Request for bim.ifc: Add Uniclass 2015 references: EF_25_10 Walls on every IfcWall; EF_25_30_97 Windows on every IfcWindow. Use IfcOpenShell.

First a look at what the model holds.

```python
import ifcopenshell

model = ifcopenshell.open("bim.ifc")
print(model.schema)
print("classifications:", [c.Name for c in model.by_type("IfcClassification")])
for ifc_class in ("IfcDoor", "IfcRoof", "IfcStair", "IfcWall", "IfcWindow"):
    print(ifc_class, len(model.by_type(ifc_class)))
```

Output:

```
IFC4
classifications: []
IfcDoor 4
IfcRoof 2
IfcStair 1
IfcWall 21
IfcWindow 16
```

```python
import ifcopenshell
import ifcopenshell.api.classification

model = ifcopenshell.open("bim.ifc")

system = ifcopenshell.api.classification.add_classification(model, classification="Uniclass 2015")

codes = {
    "IfcWall": ("EF_25_10", "Walls"),
    "IfcWindow": ("EF_25_30_97", "Windows"),
}
for ifc_class, (code, name) in codes.items():
    products = model.by_type(ifc_class)
    ifcopenshell.api.classification.add_reference(
        model, products=products, classification=system, identification=code, name=name
    )
    print(code, len(products))

model.write("bim_rev.ifc")
```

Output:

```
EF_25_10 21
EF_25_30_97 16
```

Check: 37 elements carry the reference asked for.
